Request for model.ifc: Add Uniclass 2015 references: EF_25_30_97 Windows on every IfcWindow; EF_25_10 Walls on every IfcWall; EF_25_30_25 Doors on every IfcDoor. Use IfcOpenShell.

First a look at what the model holds.

```python
import ifcopenshell

model = ifcopenshell.open("model.ifc")
print(model.schema)
print("classifications:", [c.Name for c in model.by_type("IfcClassification")])
for ifc_class in ("IfcDoor", "IfcRoof", "IfcStair", "IfcWall", "IfcWindow"):
    print(ifc_class, len(model.by_type(ifc_class)))
```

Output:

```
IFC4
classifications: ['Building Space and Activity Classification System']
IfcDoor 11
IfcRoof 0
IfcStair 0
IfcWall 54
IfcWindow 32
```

```python
import ifcopenshell
import ifcopenshell.api.classification

model = ifcopenshell.open("model.ifc")

system = ifcopenshell.api.classification.add_classification(model, classification="Uniclass 2015")

codes = {
    "IfcWindow": ("EF_25_30_97", "Windows"),
    "IfcWall": ("EF_25_10", "Walls"),
    "IfcDoor": ("EF_25_30_25", "Doors"),
}
for ifc_class, (code, name) in codes.items():
    products = model.by_type(ifc_class)
    ifcopenshell.api.classification.add_reference(
        model, products=products, classification=system, identification=code, name=name
    )
    print(code, len(products))

model.write("model_v2.ifc")
```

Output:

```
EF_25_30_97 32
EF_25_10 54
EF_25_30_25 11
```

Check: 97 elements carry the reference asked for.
